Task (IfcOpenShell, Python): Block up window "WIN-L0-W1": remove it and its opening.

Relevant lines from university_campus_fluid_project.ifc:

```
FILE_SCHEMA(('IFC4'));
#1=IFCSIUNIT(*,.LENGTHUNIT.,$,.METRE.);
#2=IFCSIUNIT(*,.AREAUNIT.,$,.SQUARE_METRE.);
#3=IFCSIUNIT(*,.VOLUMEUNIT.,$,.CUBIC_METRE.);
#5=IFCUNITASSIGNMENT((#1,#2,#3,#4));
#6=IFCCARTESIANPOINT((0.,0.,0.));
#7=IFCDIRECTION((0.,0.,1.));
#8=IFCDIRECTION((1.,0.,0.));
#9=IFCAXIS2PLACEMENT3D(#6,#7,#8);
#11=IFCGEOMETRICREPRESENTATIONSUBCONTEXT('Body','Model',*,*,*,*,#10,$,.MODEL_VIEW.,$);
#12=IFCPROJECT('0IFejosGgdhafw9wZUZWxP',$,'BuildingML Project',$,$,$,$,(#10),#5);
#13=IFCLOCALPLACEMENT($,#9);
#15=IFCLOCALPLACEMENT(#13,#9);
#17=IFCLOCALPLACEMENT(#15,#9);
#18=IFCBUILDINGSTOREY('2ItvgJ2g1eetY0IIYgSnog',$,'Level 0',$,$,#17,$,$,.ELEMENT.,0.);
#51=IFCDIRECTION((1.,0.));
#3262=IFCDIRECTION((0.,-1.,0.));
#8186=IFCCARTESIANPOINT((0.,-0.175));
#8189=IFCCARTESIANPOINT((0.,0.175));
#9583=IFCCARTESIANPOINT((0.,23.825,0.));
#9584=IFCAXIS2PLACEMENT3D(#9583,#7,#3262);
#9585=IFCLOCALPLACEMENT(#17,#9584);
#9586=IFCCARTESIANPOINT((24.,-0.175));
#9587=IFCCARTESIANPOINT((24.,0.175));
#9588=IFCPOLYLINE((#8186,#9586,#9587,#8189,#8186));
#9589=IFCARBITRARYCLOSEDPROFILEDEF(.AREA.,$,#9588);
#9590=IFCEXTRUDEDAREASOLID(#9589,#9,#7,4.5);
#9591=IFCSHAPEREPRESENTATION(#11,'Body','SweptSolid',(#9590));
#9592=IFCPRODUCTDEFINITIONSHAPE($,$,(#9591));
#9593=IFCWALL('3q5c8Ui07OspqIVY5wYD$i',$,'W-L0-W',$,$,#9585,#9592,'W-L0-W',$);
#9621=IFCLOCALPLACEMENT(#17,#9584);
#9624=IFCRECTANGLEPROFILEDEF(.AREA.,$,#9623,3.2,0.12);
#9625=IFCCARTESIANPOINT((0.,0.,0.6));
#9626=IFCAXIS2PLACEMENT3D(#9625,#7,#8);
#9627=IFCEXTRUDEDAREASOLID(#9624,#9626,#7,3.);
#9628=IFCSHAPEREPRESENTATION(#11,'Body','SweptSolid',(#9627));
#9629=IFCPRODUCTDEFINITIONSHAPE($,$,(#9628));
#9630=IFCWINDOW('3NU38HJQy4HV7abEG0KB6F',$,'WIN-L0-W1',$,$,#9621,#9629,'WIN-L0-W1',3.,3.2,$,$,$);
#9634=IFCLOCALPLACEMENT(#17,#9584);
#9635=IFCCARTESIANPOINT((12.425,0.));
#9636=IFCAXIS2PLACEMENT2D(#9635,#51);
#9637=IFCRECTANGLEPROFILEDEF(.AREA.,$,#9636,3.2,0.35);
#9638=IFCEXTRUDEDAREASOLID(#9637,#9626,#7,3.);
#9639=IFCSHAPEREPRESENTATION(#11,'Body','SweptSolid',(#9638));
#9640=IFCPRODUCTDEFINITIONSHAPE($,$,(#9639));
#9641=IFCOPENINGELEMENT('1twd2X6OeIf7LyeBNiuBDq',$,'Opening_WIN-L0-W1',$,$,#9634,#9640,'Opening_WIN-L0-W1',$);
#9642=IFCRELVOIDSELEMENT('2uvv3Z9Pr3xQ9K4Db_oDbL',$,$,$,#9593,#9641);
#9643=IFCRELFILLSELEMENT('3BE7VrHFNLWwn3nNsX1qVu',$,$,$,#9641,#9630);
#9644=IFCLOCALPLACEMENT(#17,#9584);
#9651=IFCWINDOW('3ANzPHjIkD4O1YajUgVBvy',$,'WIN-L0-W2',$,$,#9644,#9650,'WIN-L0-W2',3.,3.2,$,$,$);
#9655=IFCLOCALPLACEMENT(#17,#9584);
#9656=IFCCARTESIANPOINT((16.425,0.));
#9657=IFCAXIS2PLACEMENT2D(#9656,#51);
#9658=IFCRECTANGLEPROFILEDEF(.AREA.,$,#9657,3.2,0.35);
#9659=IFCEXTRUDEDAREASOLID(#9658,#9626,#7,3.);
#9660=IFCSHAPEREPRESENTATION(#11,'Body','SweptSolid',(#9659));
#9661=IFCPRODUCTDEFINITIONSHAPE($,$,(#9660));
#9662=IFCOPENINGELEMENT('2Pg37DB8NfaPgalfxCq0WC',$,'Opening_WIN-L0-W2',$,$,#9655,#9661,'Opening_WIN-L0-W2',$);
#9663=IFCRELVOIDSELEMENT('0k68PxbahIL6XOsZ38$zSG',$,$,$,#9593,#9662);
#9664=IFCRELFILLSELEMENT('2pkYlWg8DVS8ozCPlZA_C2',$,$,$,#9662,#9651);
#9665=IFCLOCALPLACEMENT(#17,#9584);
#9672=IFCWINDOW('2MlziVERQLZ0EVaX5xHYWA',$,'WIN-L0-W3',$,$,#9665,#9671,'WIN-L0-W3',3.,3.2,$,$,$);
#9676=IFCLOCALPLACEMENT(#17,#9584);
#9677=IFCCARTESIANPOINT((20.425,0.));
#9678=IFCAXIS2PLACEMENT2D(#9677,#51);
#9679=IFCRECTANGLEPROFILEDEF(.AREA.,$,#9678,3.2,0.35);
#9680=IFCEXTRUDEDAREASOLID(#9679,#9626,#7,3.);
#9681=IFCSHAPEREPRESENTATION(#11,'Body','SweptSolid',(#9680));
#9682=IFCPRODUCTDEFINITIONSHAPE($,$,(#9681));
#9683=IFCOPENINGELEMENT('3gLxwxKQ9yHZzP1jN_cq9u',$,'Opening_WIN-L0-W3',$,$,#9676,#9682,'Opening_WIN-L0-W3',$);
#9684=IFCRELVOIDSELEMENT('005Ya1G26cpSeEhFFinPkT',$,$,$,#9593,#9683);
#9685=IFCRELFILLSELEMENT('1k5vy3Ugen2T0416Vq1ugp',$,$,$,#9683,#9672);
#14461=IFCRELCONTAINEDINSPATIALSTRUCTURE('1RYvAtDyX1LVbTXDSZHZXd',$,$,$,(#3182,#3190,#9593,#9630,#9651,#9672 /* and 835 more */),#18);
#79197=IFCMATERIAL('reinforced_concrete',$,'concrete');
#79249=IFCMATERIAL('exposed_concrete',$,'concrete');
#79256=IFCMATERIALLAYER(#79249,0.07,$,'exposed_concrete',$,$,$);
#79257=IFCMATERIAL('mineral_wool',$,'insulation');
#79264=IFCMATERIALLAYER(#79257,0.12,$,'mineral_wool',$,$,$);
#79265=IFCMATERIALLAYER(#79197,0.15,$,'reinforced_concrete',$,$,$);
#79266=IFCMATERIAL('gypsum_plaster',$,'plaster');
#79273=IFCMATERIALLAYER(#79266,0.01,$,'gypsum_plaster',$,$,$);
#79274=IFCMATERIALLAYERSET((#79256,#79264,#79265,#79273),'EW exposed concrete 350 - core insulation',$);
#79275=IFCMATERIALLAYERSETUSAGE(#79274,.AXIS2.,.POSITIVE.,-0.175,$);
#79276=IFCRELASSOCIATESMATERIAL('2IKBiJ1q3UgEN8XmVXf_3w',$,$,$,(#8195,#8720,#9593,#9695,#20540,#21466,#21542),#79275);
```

```python
import ifcopenshell
import ifcopenshell.api.feature
import ifcopenshell.api.root
import ifcopenshell.geom
import ifcopenshell.util.shape

model = ifcopenshell.open("university_campus_fluid_project.ifc")
settings = ifcopenshell.geom.settings()


def volume(element):
    """Net volume in cubic metres, openings subtracted."""
    shape = ifcopenshell.geom.create_shape(settings, element)
    return ifcopenshell.util.shape.get_volume(shape.geometry)


window = model.by_guid("3NU38HJQy4HV7abEG0KB6F")
opening = window.FillsVoids[0].RelatingOpeningElement
wall = opening.VoidsElements[0].RelatingBuildingElement
before = volume(wall)

ifcopenshell.api.root.remove_product(model, product=window)
ifcopenshell.api.feature.remove_feature(model, feature=opening)

after = volume(wall)

print(f"wall volume {before:.3f} -> {after:.3f} m3")

model.write("university_campus_fluid_project_updated.ifc")
```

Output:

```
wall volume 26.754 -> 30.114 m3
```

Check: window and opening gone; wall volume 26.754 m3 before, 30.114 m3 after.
